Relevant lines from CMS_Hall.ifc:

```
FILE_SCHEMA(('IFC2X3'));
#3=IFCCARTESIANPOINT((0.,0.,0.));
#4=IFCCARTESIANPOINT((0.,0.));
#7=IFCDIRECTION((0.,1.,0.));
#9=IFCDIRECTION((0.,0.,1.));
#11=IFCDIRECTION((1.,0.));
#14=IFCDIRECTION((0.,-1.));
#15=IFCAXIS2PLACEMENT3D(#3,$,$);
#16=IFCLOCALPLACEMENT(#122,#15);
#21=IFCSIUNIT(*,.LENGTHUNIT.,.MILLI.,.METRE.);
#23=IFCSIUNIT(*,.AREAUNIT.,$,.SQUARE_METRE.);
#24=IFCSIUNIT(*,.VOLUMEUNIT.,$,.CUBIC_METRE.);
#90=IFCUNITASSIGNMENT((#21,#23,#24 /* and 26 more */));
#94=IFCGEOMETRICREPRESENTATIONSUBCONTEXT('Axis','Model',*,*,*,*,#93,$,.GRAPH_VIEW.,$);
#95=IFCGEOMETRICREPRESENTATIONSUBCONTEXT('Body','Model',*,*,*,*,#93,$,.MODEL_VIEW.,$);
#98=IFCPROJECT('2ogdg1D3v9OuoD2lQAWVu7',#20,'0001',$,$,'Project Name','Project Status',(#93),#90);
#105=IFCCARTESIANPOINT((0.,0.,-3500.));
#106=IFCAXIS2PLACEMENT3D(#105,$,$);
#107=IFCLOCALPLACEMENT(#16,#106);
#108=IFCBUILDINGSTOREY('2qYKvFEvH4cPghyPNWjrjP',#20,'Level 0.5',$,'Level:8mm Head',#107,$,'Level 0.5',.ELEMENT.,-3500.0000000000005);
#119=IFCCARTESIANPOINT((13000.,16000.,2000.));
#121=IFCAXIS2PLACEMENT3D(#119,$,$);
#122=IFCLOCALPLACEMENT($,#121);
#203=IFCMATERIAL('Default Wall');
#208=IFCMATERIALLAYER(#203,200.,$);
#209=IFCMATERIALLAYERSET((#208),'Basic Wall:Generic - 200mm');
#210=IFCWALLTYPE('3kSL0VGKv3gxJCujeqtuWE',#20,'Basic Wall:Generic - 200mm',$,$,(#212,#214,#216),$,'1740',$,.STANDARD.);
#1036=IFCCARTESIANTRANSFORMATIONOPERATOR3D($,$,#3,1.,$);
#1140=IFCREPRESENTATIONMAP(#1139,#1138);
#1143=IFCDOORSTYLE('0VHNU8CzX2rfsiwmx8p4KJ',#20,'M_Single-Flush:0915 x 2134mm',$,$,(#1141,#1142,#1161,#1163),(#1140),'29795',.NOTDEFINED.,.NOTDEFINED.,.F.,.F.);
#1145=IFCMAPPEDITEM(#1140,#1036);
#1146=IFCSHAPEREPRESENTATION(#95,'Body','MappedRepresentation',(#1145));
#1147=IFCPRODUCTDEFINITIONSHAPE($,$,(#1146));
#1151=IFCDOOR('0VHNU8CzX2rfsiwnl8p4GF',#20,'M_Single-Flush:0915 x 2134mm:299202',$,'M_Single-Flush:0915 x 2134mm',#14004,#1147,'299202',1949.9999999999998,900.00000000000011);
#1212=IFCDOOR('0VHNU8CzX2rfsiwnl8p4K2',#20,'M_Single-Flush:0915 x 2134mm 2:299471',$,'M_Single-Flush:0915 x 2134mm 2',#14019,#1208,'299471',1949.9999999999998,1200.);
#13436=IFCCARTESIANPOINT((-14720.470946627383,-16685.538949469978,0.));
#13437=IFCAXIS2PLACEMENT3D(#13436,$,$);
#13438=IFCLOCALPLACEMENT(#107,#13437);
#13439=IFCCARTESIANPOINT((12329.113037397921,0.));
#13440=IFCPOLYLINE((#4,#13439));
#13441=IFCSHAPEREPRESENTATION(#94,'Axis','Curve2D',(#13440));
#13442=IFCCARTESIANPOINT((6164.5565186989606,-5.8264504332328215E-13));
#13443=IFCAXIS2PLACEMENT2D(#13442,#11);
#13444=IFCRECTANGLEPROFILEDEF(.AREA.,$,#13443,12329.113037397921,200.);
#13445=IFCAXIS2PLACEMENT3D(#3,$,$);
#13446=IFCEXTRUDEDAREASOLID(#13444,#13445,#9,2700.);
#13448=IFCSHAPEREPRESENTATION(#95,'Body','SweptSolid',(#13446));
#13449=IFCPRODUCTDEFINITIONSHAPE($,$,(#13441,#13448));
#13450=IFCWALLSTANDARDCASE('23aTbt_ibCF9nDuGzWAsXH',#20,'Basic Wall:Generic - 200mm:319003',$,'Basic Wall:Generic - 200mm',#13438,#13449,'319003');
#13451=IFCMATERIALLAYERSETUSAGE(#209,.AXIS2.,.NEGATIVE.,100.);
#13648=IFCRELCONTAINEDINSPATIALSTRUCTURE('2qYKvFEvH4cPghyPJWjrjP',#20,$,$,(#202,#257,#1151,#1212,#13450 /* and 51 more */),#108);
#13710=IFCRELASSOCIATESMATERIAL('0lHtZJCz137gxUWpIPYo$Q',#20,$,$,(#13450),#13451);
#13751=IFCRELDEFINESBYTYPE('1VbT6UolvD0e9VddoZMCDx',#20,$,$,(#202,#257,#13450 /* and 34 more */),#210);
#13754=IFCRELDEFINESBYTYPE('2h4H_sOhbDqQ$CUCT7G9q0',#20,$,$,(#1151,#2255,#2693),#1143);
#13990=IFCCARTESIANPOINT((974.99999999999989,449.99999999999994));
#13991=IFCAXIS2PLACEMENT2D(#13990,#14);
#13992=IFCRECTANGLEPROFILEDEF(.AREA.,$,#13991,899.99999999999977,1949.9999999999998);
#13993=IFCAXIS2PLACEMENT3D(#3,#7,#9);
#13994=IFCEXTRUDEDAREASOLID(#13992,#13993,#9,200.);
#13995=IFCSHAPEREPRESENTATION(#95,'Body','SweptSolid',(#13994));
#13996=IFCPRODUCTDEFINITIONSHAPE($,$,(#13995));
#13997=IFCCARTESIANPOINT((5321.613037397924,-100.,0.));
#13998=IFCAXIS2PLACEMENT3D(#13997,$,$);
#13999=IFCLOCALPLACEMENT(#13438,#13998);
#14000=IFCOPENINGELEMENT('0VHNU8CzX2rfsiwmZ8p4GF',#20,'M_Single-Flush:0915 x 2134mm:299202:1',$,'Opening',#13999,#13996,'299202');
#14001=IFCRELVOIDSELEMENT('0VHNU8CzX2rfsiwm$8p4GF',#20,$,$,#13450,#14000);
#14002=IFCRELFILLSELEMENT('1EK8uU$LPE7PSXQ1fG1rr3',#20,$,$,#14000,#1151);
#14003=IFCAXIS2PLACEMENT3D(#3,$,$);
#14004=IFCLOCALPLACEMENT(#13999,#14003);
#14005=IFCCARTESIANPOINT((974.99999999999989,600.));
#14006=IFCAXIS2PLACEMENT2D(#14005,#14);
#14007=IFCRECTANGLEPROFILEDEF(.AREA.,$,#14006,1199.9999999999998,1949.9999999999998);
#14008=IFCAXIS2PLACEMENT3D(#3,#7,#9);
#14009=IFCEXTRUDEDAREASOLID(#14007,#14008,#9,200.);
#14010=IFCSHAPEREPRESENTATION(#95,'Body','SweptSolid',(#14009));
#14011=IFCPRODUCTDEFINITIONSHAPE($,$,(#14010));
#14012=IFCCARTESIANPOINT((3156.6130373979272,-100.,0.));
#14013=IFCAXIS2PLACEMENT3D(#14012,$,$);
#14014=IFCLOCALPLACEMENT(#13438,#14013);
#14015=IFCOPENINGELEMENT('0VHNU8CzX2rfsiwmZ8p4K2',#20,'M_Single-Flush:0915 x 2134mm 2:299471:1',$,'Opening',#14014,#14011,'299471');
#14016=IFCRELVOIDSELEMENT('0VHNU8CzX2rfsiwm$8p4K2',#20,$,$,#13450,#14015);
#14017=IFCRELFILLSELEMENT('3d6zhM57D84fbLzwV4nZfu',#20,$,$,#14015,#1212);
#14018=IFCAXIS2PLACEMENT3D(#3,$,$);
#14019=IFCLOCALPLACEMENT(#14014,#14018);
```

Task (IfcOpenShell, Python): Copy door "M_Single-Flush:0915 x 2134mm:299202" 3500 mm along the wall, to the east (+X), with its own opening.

```python
import ifcopenshell
import ifcopenshell.api.feature
import ifcopenshell.api.geometry
import ifcopenshell.api.root
import ifcopenshell.geom
import ifcopenshell.util.element
import ifcopenshell.util.placement
import ifcopenshell.util.shape

model = ifcopenshell.open("CMS_Hall.ifc")
settings = ifcopenshell.geom.settings()


def volume(element):
    """Net volume in cubic metres, openings subtracted."""
    shape = ifcopenshell.geom.create_shape(settings, element)
    return ifcopenshell.util.shape.get_volume(shape.geometry)


def reuse_history(source, copy):
    """copy_class also copies each property set's owner history, people and application; keep the originals."""
    for rel in copy.IsDefinedBy:
        if rel.is_a("IfcRelDefinesByProperties") and (history := rel.RelatingPropertyDefinition.OwnerHistory):
            rel.RelatingPropertyDefinition.OwnerHistory = source.OwnerHistory
            ifcopenshell.util.element.remove_deep2(model, history)


door = model.by_guid("0VHNU8CzX2rfsiwnl8p4GF")
opening = door.FillsVoids[0].RelatingOpeningElement
wall = opening.VoidsElements[0].RelatingBuildingElement
before = volume(wall)
shift = ifcopenshell.util.placement.get_local_placement(wall.ObjectPlacement)[:3, 0] * 3500.0

# copy_class copies the void relationship, type, container and properties, but no geometry.
new_opening = ifcopenshell.api.root.copy_class(model, product=opening)
new_opening.Representation = ifcopenshell.util.element.copy_deep(
    model, opening.Representation, exclude=["IfcGeometricRepresentationContext", "IfcRepresentationMap"]
)
new_opening.Name = "M_Single-Flush:0915 x 2134mm"
new_opening.Tag = None
new_door = ifcopenshell.api.root.copy_class(model, product=door)
new_door.Representation = ifcopenshell.util.element.copy_deep(
    model, door.Representation, exclude=["IfcGeometricRepresentationContext", "IfcRepresentationMap"]
)
new_door.Name = "M_Single-Flush:0915 x 2134mm"
new_door.Tag = None
reuse_history(door, new_door)
fills = ifcopenshell.api.feature.add_filling(model, opening=new_opening, element=new_door)
fills.OwnerHistory = new_door.OwnerHistory  # required in IFC2X3

for old, new in ((opening, new_opening), (door, new_door)):
    matrix = ifcopenshell.util.placement.get_local_placement(old.ObjectPlacement)
    matrix[:3, 3] += shift
    ifcopenshell.api.geometry.edit_object_placement(model, product=new, matrix=matrix, is_si=False)

after = volume(wall)

print(f"wall volume {before:.3f} -> {after:.3f} m3")

model.write("CMS_Hall_edited.ifc")
```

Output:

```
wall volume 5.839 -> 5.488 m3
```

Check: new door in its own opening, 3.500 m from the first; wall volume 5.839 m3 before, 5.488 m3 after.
